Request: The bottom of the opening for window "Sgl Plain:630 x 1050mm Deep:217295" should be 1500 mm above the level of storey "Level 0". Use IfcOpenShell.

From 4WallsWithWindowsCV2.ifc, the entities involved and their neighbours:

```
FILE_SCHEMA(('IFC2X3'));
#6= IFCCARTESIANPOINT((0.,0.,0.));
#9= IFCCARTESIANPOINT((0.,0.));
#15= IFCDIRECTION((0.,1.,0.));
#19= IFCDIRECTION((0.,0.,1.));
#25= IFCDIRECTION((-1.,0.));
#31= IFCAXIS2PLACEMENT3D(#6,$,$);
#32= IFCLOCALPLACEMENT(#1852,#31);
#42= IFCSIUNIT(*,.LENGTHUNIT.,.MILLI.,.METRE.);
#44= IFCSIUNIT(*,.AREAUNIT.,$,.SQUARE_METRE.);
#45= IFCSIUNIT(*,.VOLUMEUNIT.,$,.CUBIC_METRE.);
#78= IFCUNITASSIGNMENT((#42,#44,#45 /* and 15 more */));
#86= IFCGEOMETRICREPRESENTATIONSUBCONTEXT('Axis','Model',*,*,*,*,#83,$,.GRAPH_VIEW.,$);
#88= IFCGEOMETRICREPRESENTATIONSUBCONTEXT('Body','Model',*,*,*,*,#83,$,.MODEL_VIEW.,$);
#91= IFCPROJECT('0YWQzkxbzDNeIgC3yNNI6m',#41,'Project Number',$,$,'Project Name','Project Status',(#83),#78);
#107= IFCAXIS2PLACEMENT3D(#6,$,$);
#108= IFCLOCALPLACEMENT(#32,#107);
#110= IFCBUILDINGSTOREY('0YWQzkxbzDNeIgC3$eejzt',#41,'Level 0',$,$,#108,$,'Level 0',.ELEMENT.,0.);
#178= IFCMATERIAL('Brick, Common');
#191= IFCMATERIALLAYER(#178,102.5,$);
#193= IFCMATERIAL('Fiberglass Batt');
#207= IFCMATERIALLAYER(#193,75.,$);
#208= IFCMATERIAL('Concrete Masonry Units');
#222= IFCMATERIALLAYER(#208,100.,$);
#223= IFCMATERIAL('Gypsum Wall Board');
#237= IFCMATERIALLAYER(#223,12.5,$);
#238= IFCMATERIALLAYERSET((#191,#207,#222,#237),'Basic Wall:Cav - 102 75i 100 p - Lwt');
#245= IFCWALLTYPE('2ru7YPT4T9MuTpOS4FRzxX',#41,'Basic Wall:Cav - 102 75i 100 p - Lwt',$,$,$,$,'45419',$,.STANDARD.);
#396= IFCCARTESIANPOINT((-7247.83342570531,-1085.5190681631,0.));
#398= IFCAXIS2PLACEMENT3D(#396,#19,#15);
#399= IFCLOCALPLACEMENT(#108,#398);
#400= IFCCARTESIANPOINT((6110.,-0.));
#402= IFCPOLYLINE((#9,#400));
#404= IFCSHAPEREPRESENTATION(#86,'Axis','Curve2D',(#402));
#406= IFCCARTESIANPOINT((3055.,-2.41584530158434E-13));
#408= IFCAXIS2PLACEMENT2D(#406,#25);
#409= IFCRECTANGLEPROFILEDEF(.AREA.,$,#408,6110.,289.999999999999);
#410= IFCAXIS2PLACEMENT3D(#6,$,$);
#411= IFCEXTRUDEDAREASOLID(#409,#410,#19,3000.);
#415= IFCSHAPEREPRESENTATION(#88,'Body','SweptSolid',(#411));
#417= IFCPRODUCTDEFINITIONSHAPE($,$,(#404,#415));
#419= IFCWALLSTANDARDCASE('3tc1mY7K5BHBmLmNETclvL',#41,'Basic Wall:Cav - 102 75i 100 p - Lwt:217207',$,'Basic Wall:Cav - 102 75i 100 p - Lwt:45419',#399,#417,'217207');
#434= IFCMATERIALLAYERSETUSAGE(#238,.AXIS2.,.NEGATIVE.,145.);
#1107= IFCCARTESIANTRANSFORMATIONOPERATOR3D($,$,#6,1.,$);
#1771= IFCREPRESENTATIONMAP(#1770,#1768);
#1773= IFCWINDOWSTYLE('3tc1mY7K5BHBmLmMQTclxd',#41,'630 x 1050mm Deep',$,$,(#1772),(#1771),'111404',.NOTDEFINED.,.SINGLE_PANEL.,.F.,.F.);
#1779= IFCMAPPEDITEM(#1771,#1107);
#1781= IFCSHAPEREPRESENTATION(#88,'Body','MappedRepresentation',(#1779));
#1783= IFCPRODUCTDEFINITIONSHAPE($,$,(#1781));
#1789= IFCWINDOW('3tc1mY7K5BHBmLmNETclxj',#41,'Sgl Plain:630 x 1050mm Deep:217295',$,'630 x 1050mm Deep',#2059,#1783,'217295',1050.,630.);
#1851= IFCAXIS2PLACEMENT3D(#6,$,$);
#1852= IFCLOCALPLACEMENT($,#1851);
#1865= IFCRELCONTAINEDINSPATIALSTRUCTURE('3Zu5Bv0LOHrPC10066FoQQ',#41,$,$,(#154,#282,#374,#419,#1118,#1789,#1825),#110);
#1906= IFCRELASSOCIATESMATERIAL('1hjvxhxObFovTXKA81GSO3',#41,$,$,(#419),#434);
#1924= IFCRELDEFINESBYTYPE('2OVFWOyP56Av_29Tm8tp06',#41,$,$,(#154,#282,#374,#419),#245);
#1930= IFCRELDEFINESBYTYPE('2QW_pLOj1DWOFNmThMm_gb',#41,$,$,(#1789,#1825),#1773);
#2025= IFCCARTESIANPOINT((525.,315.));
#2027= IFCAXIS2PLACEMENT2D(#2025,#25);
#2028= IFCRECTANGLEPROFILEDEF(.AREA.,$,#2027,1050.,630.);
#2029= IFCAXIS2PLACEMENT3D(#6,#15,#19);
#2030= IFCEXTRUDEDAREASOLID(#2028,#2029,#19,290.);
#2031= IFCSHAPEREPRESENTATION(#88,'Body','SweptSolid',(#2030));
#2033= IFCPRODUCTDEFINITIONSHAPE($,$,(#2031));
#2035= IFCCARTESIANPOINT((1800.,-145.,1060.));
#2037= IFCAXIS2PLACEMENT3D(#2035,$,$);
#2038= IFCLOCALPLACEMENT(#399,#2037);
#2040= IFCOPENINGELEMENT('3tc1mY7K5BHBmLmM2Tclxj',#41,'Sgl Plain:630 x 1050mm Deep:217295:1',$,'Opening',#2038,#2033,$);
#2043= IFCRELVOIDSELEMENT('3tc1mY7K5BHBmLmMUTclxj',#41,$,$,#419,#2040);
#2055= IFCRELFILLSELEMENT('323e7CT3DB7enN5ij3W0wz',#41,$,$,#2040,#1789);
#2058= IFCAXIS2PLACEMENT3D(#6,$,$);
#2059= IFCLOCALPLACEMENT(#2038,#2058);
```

```python
import numpy as np
import ifcopenshell
import ifcopenshell.api.geometry
import ifcopenshell.geom
import ifcopenshell.util.element
import ifcopenshell.util.placement
import ifcopenshell.util.shape
import ifcopenshell.util.unit

model = ifcopenshell.open("4WallsWithWindowsCV2.ifc")
unit_scale = ifcopenshell.util.unit.calculate_unit_scale(model)

window = model.by_id(1789)
opening = window.FillsVoids[0].RelatingOpeningElement
storey = ifcopenshell.util.element.get_container(window, ifc_class="IfcBuildingStorey")
level = ifcopenshell.util.placement.get_local_placement(storey.ObjectPlacement)[2, 3]

# The opening's origin need not be at the sill, so measure its lowest point.
shape = ifcopenshell.geom.create_shape(ifcopenshell.geom.settings(), opening)
bottom = ifcopenshell.util.shape.get_shape_bottom_elevation(shape, shape.geometry) / unit_scale
dz = level + 1.5 / unit_scale - bottom

shift = np.array([0.0, 0.0, dz])
# The window is placed relative to its opening, so it follows when the opening moves.
matrix = ifcopenshell.util.placement.get_local_placement(opening.ObjectPlacement)
matrix[:3, 3] += shift
ifcopenshell.api.geometry.edit_object_placement(
    model, product=opening, matrix=matrix, is_si=False, should_transform_children=True
)

print(f"moved by {dz * unit_scale:+.3f} m")

model.write("4WallsWithWindowsCV2-out.ifc")
```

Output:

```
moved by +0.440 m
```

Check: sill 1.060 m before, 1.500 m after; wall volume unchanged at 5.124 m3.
